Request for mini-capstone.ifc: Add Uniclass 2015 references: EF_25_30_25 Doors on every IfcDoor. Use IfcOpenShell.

First a look at what the model holds.

```python
import ifcopenshell

model = ifcopenshell.open("mini-capstone.ifc")
print(model.schema)
print("classifications:", [c.Name for c in model.by_type("IfcClassification")])
for ifc_class in ("IfcDoor", "IfcRoof", "IfcStair", "IfcWall", "IfcWindow"):
    print(ifc_class, len(model.by_type(ifc_class)))
```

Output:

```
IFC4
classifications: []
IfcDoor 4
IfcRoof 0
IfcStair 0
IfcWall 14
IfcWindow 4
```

```python
import ifcopenshell
import ifcopenshell.api.classification

model = ifcopenshell.open("mini-capstone.ifc")

system = ifcopenshell.api.classification.add_classification(model, classification="Uniclass 2015")

codes = {
    "IfcDoor": ("EF_25_30_25", "Doors"),
}
for ifc_class, (code, name) in codes.items():
    products = model.by_type(ifc_class)
    ifcopenshell.api.classification.add_reference(
        model, products=products, classification=system, identification=code, name=name
    )
    print(code, len(products))

model.write("mini-capstone_edited.ifc")
```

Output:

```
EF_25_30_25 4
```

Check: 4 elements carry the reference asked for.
